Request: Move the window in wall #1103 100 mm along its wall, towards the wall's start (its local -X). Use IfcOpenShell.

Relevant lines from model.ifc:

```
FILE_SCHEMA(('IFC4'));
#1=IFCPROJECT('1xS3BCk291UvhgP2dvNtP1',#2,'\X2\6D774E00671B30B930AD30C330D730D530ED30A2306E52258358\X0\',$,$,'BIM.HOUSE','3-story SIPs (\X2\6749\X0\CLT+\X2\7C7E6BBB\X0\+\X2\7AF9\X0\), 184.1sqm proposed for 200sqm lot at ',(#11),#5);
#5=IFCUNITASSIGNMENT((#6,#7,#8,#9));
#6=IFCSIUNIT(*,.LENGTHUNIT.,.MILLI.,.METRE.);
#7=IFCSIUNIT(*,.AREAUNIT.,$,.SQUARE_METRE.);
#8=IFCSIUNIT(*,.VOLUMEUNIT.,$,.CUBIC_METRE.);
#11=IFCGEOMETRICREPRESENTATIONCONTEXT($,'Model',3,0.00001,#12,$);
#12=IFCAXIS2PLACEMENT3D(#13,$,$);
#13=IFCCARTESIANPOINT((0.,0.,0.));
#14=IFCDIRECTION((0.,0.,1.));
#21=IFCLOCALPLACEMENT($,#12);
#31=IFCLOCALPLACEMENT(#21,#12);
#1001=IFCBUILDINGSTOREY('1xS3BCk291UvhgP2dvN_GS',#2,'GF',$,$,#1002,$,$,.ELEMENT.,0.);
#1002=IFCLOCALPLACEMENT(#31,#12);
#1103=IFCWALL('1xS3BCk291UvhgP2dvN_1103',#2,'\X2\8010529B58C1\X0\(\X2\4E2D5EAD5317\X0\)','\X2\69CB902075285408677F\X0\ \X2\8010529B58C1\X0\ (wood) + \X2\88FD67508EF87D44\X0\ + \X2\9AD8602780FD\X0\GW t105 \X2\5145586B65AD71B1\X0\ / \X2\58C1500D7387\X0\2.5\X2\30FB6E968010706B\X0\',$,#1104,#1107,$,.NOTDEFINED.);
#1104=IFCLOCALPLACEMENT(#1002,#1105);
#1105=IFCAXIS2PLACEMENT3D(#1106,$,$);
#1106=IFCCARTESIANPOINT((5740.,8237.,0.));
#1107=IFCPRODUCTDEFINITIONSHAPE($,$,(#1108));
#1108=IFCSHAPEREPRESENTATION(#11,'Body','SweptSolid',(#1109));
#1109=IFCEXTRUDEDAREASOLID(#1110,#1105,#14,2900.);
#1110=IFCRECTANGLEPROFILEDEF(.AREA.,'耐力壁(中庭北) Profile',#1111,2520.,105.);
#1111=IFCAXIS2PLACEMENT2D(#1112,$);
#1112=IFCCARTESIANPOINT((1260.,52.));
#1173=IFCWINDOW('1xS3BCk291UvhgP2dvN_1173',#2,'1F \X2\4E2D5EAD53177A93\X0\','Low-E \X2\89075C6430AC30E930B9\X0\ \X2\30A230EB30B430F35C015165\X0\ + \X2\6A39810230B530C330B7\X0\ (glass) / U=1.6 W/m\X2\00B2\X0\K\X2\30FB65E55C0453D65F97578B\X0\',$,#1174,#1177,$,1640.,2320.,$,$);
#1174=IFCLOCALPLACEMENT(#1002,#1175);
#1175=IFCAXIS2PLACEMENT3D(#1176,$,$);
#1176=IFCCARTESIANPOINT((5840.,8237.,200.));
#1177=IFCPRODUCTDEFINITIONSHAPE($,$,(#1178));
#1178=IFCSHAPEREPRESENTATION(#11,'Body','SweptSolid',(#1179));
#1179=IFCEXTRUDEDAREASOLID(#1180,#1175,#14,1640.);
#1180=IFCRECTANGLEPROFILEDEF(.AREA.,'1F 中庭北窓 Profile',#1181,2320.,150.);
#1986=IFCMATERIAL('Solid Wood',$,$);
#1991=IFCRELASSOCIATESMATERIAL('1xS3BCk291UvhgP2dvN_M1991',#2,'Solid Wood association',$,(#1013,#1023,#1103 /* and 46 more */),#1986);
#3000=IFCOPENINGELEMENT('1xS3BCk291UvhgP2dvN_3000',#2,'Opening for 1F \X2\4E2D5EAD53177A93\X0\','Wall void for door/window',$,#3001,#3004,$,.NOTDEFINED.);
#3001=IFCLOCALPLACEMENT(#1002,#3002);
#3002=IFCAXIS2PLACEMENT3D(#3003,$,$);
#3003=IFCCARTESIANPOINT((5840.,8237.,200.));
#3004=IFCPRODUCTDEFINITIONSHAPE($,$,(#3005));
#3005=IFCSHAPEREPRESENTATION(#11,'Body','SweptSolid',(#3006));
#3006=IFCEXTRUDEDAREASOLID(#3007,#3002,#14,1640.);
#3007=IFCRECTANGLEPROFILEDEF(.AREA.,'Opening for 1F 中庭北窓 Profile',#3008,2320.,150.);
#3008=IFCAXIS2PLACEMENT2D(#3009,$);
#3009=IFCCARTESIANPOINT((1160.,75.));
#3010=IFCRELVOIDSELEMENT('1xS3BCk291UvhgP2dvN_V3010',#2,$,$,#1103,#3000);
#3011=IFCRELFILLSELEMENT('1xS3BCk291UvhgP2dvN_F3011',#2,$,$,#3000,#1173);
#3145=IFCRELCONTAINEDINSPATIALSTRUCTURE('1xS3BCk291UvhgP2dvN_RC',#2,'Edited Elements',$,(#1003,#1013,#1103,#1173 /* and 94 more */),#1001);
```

```python
import ifcopenshell
import ifcopenshell.api.geometry
import ifcopenshell.util.placement
import ifcopenshell.util.unit

model = ifcopenshell.open("model.ifc")
unit_scale = ifcopenshell.util.unit.calculate_unit_scale(model)

window = model.by_guid("1xS3BCk291UvhgP2dvN_1173")
opening = window.FillsVoids[0].RelatingOpeningElement
wall = opening.VoidsElements[0].RelatingBuildingElement

wall_matrix = ifcopenshell.util.placement.get_local_placement(wall.ObjectPlacement)
shift = wall_matrix[:3, 0] * -0.1 / unit_scale
before = ifcopenshell.util.placement.get_local_placement(window.ObjectPlacement)[:3, 3].copy()

# The window is not placed relative to its opening, so move both.
for product in (opening, window):
    matrix = ifcopenshell.util.placement.get_local_placement(product.ObjectPlacement)
    matrix[:3, 3] += shift
    ifcopenshell.api.geometry.edit_object_placement(model, product=product, matrix=matrix, is_si=False)

after = ifcopenshell.util.placement.get_local_placement(window.ObjectPlacement)[:3, 3]
print("window moved by", (after - before).round(3) + 0.0)

model.write("model_edited.ifc")
```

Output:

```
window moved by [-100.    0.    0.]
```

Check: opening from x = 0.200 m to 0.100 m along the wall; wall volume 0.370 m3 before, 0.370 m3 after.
